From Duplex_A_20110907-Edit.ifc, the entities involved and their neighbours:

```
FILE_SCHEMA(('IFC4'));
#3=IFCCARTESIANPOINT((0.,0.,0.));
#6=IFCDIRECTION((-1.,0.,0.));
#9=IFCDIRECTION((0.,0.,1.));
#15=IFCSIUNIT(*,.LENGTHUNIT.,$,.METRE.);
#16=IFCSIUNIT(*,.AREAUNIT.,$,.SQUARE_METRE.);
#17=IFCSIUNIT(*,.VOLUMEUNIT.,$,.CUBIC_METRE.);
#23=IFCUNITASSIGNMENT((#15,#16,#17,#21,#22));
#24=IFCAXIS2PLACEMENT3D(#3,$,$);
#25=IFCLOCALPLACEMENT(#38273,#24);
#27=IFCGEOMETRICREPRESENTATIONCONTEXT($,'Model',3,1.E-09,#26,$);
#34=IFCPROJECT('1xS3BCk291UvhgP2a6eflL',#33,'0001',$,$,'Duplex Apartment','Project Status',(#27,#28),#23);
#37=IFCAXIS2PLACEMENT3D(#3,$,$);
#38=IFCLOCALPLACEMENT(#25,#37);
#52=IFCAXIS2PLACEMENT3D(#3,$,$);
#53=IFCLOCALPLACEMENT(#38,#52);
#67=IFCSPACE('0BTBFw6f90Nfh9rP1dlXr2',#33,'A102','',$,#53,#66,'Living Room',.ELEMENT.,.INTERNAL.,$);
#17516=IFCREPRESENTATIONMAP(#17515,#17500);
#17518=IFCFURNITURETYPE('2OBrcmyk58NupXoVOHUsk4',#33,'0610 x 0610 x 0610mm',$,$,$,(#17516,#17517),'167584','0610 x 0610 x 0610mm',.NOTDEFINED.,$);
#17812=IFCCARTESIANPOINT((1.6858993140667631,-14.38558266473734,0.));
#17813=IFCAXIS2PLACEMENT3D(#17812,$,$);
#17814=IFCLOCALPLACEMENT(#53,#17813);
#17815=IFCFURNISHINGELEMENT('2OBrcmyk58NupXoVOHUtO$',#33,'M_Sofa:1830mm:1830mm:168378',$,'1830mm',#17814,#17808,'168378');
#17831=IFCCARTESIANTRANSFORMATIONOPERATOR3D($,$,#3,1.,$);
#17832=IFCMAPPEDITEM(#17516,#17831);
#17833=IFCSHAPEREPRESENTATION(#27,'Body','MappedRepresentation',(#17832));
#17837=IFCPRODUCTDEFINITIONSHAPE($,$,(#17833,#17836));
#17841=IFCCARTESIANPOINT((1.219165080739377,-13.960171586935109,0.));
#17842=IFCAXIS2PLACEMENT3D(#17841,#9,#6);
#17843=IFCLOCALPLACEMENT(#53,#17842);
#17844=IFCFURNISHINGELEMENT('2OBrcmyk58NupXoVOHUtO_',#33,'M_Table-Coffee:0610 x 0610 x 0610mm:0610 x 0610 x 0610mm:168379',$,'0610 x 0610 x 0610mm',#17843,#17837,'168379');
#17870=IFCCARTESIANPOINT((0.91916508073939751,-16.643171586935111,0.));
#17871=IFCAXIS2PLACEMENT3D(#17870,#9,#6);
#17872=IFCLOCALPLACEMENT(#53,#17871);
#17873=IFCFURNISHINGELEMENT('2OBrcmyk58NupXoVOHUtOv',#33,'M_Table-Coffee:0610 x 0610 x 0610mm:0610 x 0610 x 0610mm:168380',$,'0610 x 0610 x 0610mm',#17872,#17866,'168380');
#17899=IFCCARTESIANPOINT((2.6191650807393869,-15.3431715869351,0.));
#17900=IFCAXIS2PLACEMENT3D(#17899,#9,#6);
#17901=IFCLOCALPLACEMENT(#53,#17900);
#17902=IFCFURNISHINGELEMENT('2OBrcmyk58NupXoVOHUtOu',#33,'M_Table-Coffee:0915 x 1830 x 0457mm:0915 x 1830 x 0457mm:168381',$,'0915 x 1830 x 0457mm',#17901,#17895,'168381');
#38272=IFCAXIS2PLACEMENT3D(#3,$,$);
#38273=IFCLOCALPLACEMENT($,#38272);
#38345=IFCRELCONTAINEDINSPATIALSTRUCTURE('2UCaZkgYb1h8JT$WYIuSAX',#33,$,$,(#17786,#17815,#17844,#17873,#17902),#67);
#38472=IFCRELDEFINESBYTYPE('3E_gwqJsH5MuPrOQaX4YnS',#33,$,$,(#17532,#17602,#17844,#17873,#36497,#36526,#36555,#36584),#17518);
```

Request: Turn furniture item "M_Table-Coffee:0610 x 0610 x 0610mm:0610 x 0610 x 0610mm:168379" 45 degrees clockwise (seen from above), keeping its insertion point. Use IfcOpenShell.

```python
import ifcopenshell
import ifcopenshell.api.geometry
import ifcopenshell.util.placement

model = ifcopenshell.open("Duplex_A_20110907-Edit.ifc")

item = model.by_guid("2OBrcmyk58NupXoVOHUtO_")
matrix = ifcopenshell.util.placement.get_local_placement(item.ObjectPlacement)
matrix = matrix @ ifcopenshell.util.placement.rotation(-45, "Z")
ifcopenshell.api.geometry.edit_object_placement(model, product=item, matrix=matrix, is_si=False)

print(ifcopenshell.util.placement.get_local_placement(item.ObjectPlacement).round(3) + 0.0)

model.write("Duplex_A_20110907-Edit_v2.ifc")
```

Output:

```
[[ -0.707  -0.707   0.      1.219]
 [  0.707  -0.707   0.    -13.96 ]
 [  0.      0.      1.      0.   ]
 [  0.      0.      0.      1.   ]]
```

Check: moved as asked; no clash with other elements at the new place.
